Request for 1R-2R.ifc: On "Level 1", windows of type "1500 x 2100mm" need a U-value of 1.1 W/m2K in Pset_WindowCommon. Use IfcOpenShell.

First a look at what the model holds.

```python
import ifcopenshell
import ifcopenshell.util.element

model = ifcopenshell.open("1R-2R.ifc")
print(model.schema)
storey = next(s for s in model.by_type("IfcBuildingStorey") if s.Name == "Level 1")
windows = [e for e in ifcopenshell.util.element.get_decomposition(storey) if e.is_a("IfcWindow")]
seen = {}
for e in windows:
    element_type = ifcopenshell.util.element.get_type(e)
    key = (element_type.Name if element_type != e and element_type else None, ifcopenshell.util.element.get_pset(e, "Pset_WindowCommon", "ThermalTransmittance"))
    seen[key] = seen.get(key, 0) + 1
for (name, value), count in sorted(seen.items(), key=str):
    print(count, "x", name, "|", value)
```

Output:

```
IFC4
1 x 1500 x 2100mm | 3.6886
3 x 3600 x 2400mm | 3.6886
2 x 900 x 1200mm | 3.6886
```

```python
import ifcopenshell
import ifcopenshell.api.pset
import ifcopenshell.util.element

model = ifcopenshell.open("1R-2R.ifc")

storey = next(s for s in model.by_type("IfcBuildingStorey") if s.Name == "Level 1")
windows = [e for e in ifcopenshell.util.element.get_decomposition(storey) if e.is_a("IfcWindow")]

count = 0
for e in windows:
    element_type = ifcopenshell.util.element.get_type(e)
    if element_type in (None, e) or element_type.Name != "1500 x 2100mm":
        continue
    # add_pset returns the element's existing set when there is one.
    pset = ifcopenshell.api.pset.add_pset(model, product=e, name="Pset_WindowCommon")
    ifcopenshell.api.pset.edit_pset(model, pset=pset, properties={"ThermalTransmittance": 1.1})
    count += 1

print(count, "windows updated")

model.write("1R-2R_rev.ifc")
```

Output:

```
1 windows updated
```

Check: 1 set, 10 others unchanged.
